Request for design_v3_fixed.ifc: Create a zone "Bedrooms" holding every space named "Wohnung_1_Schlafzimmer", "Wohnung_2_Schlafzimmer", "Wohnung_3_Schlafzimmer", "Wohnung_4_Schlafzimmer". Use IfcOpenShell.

First a look at what the model holds.

```python
import ifcopenshell

model = ifcopenshell.open("design_v3_fixed.ifc")
print(model.schema)
seen = {}
for space in model.by_type("IfcSpace"):
    seen[space.LongName] = seen.get(space.LongName, 0) + 1
for name, count in sorted(seen.items(), key=str):
    print(count, "x", name)
print("zones:", [z.Name for z in model.by_type("IfcZone")][:20])
```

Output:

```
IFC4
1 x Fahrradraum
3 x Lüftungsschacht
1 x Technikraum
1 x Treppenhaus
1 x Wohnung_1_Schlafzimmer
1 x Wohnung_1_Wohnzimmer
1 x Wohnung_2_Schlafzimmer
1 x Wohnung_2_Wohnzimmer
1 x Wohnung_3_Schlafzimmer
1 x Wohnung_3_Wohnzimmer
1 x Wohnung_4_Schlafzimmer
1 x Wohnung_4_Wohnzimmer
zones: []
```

```python
import ifcopenshell
import ifcopenshell.api.group
import ifcopenshell.api.root

model = ifcopenshell.open("design_v3_fixed.ifc")

names = {"Wohnung_1_Schlafzimmer", "Wohnung_2_Schlafzimmer", "Wohnung_3_Schlafzimmer", "Wohnung_4_Schlafzimmer"}
spaces = [s for s in model.by_type("IfcSpace") if s.LongName in names]

zone = ifcopenshell.api.root.create_entity(model, ifc_class="IfcZone", name="Bedrooms")
ifcopenshell.api.group.assign_group(model, products=spaces, group=zone)
print(len(spaces), "spaces in", zone.Name)

model.write("design_v3_fixed_rev.ifc")
```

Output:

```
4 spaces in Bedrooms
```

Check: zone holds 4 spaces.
